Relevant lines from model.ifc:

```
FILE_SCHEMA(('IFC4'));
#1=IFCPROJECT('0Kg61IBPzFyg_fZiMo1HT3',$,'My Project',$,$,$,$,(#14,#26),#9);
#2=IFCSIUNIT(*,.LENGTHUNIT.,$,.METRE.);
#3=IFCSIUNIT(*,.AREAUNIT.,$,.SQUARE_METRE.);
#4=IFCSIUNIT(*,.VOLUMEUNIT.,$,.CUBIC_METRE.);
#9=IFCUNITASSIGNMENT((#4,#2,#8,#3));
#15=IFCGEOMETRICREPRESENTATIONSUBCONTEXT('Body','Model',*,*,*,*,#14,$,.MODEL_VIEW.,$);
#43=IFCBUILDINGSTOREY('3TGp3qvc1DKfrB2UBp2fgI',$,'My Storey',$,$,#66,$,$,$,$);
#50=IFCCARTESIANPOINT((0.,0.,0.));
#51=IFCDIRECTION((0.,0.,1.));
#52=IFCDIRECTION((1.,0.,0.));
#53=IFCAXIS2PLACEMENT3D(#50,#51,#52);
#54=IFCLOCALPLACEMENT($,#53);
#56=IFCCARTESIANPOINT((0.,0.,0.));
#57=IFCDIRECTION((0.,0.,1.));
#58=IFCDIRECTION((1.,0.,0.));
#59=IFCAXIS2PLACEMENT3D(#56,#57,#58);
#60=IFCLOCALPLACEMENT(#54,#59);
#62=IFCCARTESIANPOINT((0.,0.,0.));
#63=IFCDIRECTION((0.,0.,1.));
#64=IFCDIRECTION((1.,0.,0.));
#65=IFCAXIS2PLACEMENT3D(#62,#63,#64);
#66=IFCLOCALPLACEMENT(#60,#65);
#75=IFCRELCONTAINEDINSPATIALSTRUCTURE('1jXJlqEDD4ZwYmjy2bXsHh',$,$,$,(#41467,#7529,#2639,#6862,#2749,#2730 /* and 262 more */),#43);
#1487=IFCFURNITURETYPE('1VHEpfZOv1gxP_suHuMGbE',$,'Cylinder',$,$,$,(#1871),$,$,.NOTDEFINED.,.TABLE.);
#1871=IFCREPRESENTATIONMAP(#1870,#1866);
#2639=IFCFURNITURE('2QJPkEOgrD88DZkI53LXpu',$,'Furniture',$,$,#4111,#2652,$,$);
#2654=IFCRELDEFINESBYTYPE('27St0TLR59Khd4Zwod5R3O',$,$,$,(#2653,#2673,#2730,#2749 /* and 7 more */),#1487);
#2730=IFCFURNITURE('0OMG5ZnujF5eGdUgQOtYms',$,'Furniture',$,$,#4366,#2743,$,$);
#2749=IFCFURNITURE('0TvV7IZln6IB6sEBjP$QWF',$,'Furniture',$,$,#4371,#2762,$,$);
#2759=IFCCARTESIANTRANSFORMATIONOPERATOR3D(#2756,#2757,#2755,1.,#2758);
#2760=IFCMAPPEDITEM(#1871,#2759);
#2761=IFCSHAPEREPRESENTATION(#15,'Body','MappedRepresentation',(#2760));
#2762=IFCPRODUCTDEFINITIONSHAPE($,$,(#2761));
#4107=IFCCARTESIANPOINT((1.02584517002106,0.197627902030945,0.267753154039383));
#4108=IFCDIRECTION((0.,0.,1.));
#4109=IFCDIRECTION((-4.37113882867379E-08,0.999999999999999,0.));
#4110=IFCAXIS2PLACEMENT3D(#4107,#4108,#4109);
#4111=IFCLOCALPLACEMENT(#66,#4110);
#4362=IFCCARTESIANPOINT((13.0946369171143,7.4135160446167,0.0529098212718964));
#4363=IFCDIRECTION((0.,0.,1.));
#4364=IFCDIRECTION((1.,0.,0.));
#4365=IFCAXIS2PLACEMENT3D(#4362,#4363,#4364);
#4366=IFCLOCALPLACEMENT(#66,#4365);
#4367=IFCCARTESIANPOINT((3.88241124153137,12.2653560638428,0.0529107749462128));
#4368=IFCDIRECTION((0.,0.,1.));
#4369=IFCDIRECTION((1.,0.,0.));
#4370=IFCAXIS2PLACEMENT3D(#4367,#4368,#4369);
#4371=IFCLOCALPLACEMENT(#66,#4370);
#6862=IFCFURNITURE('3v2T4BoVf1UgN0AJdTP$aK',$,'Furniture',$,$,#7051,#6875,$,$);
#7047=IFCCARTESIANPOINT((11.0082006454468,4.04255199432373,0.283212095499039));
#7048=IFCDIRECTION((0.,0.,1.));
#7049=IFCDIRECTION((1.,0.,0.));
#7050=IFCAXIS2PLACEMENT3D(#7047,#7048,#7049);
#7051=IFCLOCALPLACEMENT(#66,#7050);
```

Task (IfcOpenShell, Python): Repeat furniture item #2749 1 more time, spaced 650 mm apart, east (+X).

```python
import numpy as np
import ifcopenshell
import ifcopenshell.api.geometry
import ifcopenshell.api.root
import ifcopenshell.util.element
import ifcopenshell.util.placement

model = ifcopenshell.open("model.ifc")

source = model.by_id(2749)
base = ifcopenshell.util.placement.get_local_placement(source.ObjectPlacement)
step = np.array([1.0, 0.0, 0.0]) * 0.65

for i in range(1, 2):
    copy = ifcopenshell.api.root.copy_class(model, product=source)
    copy.Representation = ifcopenshell.util.element.copy_deep(
        model, source.Representation, exclude=["IfcGeometricRepresentationContext", "IfcRepresentationMap"]
    )
    matrix = base.copy()
    matrix[:3, 3] += i * step
    print("added at", matrix[:3, 3].round(3) + 0.0)
    ifcopenshell.api.geometry.edit_object_placement(model, product=copy, matrix=matrix, is_si=False)

model.write("model_v2.ifc")
```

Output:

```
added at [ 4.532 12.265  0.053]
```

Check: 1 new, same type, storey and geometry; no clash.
